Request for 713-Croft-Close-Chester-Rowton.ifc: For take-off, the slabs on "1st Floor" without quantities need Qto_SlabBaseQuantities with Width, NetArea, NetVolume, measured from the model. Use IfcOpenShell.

First a look at what the model holds.

```python
import ifcopenshell
import ifcopenshell.util.element
import ifcopenshell.util.unit

model = ifcopenshell.open("713-Croft-Close-Chester-Rowton.ifc")
print(model.schema)
for unit_type in ("LENGTHUNIT", "AREAUNIT", "VOLUMEUNIT"):
    print(unit_type, ifcopenshell.util.unit.calculate_unit_scale(model, unit_type))
storey = next(s for s in model.by_type("IfcBuildingStorey") if s.Name == "1st Floor")
slabs = [e for e in ifcopenshell.util.element.get_decomposition(storey) if e.is_a("IfcSlab")]
for e in sorted(slabs, key=lambda e: e.id()):
    print(e.id(), e.is_a(), e.Name, list(ifcopenshell.util.element.get_psets(e, qtos_only=True)), sep=" | ")
```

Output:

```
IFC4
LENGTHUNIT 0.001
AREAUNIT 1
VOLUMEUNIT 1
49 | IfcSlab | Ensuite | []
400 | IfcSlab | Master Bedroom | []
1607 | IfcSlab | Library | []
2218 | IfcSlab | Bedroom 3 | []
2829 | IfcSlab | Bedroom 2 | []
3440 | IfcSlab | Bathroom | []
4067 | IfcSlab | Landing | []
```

```python
import ifcopenshell
import ifcopenshell.api.pset
import ifcopenshell.geom
import ifcopenshell.util.element
import ifcopenshell.util.shape
import ifcopenshell.util.unit

model = ifcopenshell.open("713-Croft-Close-Chester-Rowton.ifc")
unit_scale = ifcopenshell.util.unit.calculate_unit_scale(model)
area_scale = ifcopenshell.util.unit.calculate_unit_scale(model, "AREAUNIT")
volume_scale = ifcopenshell.util.unit.calculate_unit_scale(model, "VOLUMEUNIT")
settings = ifcopenshell.geom.settings()

storey = next(s for s in model.by_type("IfcBuildingStorey") if s.Name == "1st Floor")
slabs = [e for e in ifcopenshell.util.element.get_decomposition(storey) if e.is_a("IfcSlab")]

for e in sorted(slabs, key=lambda e: e.id()):
    if ifcopenshell.util.element.get_psets(e, qtos_only=True, should_inherit=False):
        continue
    # Geometry comes back in metres, in the element's own axes.
    shape = ifcopenshell.geom.create_shape(settings, e)
    values = {
        "Width": ifcopenshell.util.shape.get_z(shape.geometry) / unit_scale,
        "NetArea": ifcopenshell.util.shape.get_footprint_area(shape.geometry) / area_scale,
        "NetVolume": ifcopenshell.util.shape.get_volume(shape.geometry) / volume_scale,
    }
    qto = ifcopenshell.api.pset.add_qto(model, product=e, name="Qto_SlabBaseQuantities")
    ifcopenshell.api.pset.edit_qto(model, qto=qto, properties=values)
    print(e.id(), {k: round(v, 3) for k, v in values.items()})

model.write("713-Croft-Close-Chester-Rowton-out.ifc")
```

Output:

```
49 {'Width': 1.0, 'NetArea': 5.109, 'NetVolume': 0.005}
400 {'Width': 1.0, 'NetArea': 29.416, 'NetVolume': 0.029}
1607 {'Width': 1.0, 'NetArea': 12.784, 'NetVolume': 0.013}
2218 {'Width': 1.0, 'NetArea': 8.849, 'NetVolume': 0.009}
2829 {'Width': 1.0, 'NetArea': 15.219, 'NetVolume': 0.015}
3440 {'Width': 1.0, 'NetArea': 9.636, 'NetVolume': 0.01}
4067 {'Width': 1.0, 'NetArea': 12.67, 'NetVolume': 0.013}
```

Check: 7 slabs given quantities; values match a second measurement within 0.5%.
